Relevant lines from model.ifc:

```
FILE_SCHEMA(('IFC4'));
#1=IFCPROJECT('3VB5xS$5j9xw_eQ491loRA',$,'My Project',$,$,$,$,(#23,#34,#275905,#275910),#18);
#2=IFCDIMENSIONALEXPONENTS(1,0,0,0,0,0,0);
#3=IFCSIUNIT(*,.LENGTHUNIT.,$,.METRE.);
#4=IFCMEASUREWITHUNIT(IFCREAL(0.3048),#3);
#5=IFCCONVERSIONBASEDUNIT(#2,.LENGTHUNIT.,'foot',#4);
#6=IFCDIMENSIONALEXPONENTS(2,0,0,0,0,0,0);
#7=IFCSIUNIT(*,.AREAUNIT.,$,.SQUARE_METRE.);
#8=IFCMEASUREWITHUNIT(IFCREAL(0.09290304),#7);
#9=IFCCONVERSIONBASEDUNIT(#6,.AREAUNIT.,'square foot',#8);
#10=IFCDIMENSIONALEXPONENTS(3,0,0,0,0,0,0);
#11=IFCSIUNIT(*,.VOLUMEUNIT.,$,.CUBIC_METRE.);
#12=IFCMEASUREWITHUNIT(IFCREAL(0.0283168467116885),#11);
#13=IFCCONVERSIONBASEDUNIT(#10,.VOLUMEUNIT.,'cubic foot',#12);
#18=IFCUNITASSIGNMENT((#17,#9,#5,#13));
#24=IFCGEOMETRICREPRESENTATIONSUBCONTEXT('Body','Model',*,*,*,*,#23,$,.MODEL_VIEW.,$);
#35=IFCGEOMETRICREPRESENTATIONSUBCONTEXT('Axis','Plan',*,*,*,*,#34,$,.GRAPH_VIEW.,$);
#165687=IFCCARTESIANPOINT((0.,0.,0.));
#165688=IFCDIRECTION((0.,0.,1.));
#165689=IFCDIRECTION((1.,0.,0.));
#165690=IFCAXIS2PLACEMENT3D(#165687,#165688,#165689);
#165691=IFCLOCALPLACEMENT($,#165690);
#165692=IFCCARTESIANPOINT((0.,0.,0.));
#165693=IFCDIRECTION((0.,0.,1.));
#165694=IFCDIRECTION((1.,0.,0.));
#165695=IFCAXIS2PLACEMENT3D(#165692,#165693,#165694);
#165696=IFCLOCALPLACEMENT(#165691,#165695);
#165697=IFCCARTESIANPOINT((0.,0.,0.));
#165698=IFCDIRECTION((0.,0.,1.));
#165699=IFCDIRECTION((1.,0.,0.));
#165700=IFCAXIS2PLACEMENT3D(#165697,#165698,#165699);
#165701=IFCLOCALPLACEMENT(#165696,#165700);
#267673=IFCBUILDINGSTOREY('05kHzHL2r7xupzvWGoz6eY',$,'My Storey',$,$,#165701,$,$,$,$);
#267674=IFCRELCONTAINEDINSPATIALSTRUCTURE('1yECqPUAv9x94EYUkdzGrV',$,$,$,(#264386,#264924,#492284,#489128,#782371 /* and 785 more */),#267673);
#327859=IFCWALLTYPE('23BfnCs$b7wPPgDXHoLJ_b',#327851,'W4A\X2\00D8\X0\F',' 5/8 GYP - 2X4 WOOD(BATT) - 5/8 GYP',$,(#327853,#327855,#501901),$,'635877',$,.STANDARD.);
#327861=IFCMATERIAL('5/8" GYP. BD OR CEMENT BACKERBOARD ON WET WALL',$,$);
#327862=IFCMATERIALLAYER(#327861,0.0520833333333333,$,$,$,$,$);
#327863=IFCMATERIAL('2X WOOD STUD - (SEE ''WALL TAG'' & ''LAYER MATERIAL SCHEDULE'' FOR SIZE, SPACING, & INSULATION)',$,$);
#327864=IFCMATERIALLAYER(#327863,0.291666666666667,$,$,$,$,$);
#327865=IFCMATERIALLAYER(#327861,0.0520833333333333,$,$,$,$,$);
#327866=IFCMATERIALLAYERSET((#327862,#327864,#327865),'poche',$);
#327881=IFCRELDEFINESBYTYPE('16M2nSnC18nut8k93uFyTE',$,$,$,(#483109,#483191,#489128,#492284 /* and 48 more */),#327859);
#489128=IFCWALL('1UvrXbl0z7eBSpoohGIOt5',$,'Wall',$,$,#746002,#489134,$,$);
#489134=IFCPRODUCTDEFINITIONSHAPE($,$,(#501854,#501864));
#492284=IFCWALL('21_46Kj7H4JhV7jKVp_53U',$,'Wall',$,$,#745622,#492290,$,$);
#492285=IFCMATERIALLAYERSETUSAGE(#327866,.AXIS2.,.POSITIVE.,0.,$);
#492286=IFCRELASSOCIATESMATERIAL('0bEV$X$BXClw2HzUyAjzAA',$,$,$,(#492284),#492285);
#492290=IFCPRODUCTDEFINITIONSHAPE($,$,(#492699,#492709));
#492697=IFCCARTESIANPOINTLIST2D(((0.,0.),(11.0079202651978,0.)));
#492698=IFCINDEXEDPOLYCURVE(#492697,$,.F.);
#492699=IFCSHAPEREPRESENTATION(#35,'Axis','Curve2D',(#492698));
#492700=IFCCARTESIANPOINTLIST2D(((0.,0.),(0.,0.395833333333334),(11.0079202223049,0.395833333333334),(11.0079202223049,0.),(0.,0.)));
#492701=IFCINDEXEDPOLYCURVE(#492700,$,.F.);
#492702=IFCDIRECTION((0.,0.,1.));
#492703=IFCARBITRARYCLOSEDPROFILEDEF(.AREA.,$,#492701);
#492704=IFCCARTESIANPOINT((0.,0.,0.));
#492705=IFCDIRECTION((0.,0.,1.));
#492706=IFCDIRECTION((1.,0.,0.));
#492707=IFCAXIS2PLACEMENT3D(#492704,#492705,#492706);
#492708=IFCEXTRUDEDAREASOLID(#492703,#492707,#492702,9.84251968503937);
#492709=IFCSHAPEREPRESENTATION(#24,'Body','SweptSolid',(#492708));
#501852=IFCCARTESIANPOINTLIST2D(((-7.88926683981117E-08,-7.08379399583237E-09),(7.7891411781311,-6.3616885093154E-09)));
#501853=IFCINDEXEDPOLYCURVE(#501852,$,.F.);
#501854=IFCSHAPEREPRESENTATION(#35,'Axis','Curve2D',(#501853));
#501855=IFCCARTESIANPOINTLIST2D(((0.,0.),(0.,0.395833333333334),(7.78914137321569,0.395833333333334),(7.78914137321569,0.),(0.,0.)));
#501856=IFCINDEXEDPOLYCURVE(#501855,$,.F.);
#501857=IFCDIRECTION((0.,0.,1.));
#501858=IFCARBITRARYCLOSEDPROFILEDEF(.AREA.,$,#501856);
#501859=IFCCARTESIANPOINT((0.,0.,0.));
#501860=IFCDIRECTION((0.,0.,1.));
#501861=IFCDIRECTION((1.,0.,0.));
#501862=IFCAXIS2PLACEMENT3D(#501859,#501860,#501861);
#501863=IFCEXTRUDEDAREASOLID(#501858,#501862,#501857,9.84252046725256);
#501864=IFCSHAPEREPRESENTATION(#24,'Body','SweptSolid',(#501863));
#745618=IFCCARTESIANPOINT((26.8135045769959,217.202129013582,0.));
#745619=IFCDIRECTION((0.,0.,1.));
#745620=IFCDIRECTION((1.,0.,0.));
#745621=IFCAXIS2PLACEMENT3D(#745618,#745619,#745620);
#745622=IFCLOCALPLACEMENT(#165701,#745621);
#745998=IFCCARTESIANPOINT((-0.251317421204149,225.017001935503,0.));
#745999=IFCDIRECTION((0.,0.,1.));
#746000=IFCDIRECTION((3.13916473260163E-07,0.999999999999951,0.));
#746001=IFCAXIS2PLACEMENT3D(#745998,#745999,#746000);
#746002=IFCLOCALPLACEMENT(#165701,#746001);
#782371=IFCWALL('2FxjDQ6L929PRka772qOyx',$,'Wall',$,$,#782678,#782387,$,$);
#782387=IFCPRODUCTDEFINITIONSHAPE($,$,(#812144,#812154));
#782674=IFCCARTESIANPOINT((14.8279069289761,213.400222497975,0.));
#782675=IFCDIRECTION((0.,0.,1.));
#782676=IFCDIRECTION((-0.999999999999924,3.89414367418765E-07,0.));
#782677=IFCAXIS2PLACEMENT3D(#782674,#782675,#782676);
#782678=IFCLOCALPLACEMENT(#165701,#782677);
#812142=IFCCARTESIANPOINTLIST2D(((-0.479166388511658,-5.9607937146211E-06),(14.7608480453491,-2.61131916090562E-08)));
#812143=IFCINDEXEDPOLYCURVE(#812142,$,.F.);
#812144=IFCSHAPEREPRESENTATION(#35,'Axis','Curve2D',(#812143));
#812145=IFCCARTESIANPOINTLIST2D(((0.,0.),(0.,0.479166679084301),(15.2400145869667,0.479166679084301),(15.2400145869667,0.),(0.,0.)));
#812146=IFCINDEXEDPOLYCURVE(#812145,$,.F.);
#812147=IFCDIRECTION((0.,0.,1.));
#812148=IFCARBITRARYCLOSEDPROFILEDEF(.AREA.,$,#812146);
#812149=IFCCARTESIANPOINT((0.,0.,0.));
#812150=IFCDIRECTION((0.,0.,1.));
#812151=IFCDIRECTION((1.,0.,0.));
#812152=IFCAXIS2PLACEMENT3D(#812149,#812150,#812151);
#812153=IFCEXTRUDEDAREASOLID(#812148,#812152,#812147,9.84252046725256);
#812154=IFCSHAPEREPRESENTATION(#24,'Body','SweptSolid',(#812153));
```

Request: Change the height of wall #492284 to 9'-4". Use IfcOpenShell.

```python
import ifcopenshell
import ifcopenshell.geom
import ifcopenshell.util.representation
import ifcopenshell.util.shape
import ifcopenshell.util.unit

model = ifcopenshell.open("model.ifc")
unit_scale = ifcopenshell.util.unit.calculate_unit_scale(model)
settings = ifcopenshell.geom.settings()


def volume(element):
    """Net volume in cubic metres, openings subtracted."""
    shape = ifcopenshell.geom.create_shape(settings, element)
    return ifcopenshell.util.shape.get_volume(shape.geometry)


wall = model.by_guid("21_46Kj7H4JhV7jKVp_53U")
before = volume(wall)

body = ifcopenshell.util.representation.get_representation(wall, "Model", "Body")
solid = body.Items[0]
old_height = solid.Depth
solid.Depth = 112 * 0.0254 / unit_scale
after = volume(wall)

print(f"height {old_height:g} -> {solid.Depth:g}, volume {before:.3f} -> {after:.3f} m3")

model.write("model_rev.ifc")
```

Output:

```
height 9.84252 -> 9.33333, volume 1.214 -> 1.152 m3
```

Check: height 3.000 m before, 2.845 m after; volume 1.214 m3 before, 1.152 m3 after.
